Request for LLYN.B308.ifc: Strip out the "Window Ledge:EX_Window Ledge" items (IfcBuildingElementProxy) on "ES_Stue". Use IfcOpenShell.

First a look at what the model holds.

```python
import ifcopenshell
import ifcopenshell.util.element

model = ifcopenshell.open("LLYN.B308.ifc")
print(model.schema)
storey = next(s for s in model.by_type("IfcBuildingStorey") if s.Name == "ES_Stue")
proxies = [e for e in ifcopenshell.util.element.get_decomposition(storey) if e.is_a("IfcBuildingElementProxy")]
seen = {}
for e in proxies:
    element_type = ifcopenshell.util.element.get_type(e)
    name = element_type.Name if element_type not in (None, e) else None
    seen[name] = seen.get(name, 0) + 1
for name, count in sorted(seen.items(), key=str):
    print(count, "x", name)
```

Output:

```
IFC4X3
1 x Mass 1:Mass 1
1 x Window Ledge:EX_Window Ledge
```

```python
import ifcopenshell
import ifcopenshell.api.root
import ifcopenshell.util.element

model = ifcopenshell.open("LLYN.B308.ifc")

storey = next(s for s in model.by_type("IfcBuildingStorey") if s.Name == "ES_Stue")
proxies = [e for e in ifcopenshell.util.element.get_decomposition(storey) if e.is_a("IfcBuildingElementProxy")]
targets = [e for e in proxies if (t := ifcopenshell.util.element.get_type(e)) not in (None, e) and t.Name == "Window Ledge:EX_Window Ledge"]

for e in targets:
    ifcopenshell.api.root.remove_product(model, product=e)
print(len(targets), "removed")

model.write("LLYN.B308_edited.ifc")
```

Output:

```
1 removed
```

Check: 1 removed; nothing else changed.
